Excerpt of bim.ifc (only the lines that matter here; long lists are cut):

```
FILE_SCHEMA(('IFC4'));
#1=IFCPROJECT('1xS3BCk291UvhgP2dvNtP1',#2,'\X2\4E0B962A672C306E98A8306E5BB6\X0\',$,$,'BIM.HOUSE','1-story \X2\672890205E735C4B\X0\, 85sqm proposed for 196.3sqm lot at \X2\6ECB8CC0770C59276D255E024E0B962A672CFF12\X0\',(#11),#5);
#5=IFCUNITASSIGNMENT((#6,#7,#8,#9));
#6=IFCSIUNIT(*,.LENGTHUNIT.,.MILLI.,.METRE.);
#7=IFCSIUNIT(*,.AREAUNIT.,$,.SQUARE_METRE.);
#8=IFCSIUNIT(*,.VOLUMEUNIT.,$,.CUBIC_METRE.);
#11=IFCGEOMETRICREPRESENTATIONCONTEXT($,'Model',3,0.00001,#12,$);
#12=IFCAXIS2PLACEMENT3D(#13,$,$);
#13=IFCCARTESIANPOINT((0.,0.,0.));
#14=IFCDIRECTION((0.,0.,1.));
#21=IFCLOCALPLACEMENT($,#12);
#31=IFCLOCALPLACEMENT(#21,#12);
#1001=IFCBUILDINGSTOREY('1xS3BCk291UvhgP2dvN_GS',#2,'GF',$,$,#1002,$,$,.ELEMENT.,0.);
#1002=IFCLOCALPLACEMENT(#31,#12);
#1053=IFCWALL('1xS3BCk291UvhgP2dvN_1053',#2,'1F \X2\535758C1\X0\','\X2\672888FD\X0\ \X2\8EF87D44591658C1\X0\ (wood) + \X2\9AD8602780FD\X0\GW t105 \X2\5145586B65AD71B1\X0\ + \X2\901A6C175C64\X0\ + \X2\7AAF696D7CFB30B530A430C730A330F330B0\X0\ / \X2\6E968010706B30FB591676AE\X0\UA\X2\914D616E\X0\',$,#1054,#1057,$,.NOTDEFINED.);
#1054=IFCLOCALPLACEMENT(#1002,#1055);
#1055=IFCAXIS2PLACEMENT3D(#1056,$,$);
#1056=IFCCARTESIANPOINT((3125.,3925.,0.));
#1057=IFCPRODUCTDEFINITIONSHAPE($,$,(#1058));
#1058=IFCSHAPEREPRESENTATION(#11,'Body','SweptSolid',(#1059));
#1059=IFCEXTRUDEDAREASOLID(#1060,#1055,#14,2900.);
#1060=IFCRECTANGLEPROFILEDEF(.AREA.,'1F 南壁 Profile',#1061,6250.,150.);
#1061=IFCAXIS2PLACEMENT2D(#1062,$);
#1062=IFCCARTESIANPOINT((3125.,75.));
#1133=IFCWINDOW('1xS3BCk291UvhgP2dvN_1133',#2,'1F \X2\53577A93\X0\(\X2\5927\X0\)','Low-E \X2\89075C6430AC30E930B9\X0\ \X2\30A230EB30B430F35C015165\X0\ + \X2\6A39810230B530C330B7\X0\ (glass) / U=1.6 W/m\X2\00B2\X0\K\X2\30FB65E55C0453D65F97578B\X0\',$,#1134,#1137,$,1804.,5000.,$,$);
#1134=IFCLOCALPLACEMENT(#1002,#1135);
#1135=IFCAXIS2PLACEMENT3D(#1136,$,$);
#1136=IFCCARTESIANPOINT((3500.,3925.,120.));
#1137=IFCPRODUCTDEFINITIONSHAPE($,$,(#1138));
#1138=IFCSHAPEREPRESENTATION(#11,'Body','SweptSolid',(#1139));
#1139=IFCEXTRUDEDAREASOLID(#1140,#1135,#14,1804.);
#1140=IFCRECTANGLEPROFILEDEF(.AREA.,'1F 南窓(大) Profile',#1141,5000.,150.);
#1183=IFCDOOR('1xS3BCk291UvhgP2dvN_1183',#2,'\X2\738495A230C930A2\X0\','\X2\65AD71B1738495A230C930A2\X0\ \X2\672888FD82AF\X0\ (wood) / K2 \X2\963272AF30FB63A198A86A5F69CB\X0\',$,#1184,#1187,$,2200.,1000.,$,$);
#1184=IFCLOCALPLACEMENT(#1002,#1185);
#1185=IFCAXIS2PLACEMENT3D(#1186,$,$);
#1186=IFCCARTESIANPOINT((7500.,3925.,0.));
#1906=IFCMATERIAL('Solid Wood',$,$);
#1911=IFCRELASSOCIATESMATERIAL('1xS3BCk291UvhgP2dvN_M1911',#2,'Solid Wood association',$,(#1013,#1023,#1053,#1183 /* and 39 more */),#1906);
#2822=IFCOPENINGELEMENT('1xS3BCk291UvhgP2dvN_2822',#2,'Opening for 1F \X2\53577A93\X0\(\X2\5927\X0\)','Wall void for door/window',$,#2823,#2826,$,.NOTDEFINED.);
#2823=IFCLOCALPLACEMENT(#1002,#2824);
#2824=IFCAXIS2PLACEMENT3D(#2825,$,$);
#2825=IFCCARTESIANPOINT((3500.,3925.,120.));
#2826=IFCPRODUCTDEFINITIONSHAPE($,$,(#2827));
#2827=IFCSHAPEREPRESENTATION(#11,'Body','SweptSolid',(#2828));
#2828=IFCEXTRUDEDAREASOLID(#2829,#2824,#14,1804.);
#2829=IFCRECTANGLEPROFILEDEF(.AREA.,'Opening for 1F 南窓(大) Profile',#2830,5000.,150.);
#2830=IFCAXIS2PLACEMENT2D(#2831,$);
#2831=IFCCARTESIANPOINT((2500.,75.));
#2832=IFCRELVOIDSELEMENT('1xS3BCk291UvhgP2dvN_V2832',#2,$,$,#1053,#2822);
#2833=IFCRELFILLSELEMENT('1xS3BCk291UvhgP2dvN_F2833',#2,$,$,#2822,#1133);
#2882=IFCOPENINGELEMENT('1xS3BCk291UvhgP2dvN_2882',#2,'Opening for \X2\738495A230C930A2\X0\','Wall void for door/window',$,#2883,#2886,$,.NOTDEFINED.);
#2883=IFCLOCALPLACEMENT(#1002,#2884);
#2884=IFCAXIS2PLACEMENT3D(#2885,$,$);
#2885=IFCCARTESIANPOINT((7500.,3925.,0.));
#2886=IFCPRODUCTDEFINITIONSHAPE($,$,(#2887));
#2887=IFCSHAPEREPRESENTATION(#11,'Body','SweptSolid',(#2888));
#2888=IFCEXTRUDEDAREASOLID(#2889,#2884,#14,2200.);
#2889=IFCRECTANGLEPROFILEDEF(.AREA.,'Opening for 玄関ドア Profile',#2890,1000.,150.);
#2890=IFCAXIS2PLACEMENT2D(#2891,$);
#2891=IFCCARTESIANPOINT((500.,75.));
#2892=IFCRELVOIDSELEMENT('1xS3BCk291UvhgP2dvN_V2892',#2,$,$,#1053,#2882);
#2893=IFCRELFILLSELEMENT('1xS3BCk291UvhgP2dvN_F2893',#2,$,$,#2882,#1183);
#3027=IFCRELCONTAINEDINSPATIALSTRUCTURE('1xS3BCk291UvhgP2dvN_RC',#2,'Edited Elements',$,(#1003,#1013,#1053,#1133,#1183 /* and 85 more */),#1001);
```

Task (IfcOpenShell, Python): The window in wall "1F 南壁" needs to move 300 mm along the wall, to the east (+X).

```python
import ifcopenshell
import ifcopenshell.api.geometry
import ifcopenshell.util.placement
import ifcopenshell.util.unit

model = ifcopenshell.open("bim.ifc")
unit_scale = ifcopenshell.util.unit.calculate_unit_scale(model)

window = model.by_guid("1xS3BCk291UvhgP2dvN_1133")
opening = window.FillsVoids[0].RelatingOpeningElement
wall = opening.VoidsElements[0].RelatingBuildingElement

wall_matrix = ifcopenshell.util.placement.get_local_placement(wall.ObjectPlacement)
shift = wall_matrix[:3, 0] * 0.3 / unit_scale
before = ifcopenshell.util.placement.get_local_placement(window.ObjectPlacement)[:3, 3].copy()

# The window is not placed relative to its opening, so move both.
for product in (opening, window):
    matrix = ifcopenshell.util.placement.get_local_placement(product.ObjectPlacement)
    matrix[:3, 3] += shift
    ifcopenshell.api.geometry.edit_object_placement(model, product=product, matrix=matrix, is_si=False)

after = ifcopenshell.util.placement.get_local_placement(window.ObjectPlacement)[:3, 3]
print("window moved by", (after - before).round(3) + 0.0)

model.write("bim_rev.ifc")
```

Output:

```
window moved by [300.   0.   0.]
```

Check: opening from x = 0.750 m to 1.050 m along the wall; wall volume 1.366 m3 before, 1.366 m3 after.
